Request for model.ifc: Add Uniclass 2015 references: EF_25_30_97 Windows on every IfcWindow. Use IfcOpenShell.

First a look at what the model holds.

```python
import ifcopenshell

model = ifcopenshell.open("model.ifc")
print(model.schema)
print("classifications:", [c.Name for c in model.by_type("IfcClassification")])
for ifc_class in ("IfcDoor", "IfcRoof", "IfcStair", "IfcWall", "IfcWindow"):
    print(ifc_class, len(model.by_type(ifc_class)))
```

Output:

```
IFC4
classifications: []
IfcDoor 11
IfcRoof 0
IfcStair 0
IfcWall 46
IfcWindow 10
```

```python
import ifcopenshell
import ifcopenshell.api.classification

model = ifcopenshell.open("model.ifc")

system = ifcopenshell.api.classification.add_classification(model, classification="Uniclass 2015")

codes = {
    "IfcWindow": ("EF_25_30_97", "Windows"),
}
for ifc_class, (code, name) in codes.items():
    products = model.by_type(ifc_class)
    ifcopenshell.api.classification.add_reference(
        model, products=products, classification=system, identification=code, name=name
    )
    print(code, len(products))

model.write("model_edited.ifc")
```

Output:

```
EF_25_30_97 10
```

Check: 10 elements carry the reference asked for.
